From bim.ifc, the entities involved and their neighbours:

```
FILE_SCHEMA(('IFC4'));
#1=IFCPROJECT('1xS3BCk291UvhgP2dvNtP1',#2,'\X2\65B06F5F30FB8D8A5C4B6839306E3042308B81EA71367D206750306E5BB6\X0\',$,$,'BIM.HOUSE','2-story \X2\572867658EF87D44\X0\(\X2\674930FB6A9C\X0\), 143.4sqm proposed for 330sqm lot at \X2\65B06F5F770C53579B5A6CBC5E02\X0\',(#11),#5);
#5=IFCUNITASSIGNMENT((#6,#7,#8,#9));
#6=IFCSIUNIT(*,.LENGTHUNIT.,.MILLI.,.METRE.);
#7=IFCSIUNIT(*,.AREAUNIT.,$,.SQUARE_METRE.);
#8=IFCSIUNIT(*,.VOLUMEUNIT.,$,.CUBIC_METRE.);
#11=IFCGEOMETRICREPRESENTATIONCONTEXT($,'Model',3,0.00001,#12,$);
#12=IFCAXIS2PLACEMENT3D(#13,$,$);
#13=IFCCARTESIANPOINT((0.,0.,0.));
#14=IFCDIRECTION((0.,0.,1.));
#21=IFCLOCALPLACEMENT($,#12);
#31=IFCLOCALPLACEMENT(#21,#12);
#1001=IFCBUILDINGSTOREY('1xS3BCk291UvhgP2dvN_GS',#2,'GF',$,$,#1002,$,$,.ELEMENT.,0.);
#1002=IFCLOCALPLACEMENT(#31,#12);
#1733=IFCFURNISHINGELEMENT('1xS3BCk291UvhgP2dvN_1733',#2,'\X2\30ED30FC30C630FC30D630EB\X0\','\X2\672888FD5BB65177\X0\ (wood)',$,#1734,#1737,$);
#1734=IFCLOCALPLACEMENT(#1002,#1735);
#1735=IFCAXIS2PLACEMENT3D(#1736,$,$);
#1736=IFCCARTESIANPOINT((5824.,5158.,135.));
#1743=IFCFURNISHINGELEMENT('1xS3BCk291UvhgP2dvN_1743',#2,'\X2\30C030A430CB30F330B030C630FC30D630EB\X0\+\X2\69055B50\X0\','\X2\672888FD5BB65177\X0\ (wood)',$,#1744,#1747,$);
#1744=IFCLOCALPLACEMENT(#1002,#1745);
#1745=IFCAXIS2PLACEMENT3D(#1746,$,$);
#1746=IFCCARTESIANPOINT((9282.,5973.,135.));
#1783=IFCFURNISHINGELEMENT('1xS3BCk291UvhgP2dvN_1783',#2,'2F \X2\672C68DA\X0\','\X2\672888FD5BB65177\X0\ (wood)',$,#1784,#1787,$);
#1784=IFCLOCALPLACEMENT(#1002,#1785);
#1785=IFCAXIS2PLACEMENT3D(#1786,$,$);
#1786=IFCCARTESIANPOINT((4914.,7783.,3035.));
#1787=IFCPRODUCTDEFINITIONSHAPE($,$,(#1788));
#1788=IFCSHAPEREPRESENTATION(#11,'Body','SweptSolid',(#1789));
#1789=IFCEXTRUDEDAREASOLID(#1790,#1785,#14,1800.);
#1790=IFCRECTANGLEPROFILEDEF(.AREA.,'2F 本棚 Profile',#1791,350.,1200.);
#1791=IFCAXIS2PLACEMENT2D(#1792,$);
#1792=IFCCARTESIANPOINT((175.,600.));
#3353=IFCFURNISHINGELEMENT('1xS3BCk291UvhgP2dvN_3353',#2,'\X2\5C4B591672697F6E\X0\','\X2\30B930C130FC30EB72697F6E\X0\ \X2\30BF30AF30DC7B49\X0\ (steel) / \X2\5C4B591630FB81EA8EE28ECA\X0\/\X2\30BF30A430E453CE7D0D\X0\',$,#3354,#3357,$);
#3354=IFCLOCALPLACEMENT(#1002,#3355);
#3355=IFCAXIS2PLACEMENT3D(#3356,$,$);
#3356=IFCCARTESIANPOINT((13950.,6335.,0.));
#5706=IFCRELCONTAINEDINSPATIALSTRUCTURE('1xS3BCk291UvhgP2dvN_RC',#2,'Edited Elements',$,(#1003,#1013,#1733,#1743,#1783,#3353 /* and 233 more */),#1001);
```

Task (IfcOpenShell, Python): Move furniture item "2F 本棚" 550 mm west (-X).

```python
import ifcopenshell
import ifcopenshell.api.geometry
import ifcopenshell.util.placement
import ifcopenshell.util.unit

model = ifcopenshell.open("bim.ifc")
unit_scale = ifcopenshell.util.unit.calculate_unit_scale(model)

item = model.by_id(1783)
matrix = ifcopenshell.util.placement.get_local_placement(item.ObjectPlacement)
matrix[0, 3] -= 0.55 / unit_scale
ifcopenshell.api.geometry.edit_object_placement(model, product=item, matrix=matrix, is_si=False)

print(ifcopenshell.util.placement.get_local_placement(item.ObjectPlacement).round(3) + 0.0)

model.write("bim_rev.ifc")
```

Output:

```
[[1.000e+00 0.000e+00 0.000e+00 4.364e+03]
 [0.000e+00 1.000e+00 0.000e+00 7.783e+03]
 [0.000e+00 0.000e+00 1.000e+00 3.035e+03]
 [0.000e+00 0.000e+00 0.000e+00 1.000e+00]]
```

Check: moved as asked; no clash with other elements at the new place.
